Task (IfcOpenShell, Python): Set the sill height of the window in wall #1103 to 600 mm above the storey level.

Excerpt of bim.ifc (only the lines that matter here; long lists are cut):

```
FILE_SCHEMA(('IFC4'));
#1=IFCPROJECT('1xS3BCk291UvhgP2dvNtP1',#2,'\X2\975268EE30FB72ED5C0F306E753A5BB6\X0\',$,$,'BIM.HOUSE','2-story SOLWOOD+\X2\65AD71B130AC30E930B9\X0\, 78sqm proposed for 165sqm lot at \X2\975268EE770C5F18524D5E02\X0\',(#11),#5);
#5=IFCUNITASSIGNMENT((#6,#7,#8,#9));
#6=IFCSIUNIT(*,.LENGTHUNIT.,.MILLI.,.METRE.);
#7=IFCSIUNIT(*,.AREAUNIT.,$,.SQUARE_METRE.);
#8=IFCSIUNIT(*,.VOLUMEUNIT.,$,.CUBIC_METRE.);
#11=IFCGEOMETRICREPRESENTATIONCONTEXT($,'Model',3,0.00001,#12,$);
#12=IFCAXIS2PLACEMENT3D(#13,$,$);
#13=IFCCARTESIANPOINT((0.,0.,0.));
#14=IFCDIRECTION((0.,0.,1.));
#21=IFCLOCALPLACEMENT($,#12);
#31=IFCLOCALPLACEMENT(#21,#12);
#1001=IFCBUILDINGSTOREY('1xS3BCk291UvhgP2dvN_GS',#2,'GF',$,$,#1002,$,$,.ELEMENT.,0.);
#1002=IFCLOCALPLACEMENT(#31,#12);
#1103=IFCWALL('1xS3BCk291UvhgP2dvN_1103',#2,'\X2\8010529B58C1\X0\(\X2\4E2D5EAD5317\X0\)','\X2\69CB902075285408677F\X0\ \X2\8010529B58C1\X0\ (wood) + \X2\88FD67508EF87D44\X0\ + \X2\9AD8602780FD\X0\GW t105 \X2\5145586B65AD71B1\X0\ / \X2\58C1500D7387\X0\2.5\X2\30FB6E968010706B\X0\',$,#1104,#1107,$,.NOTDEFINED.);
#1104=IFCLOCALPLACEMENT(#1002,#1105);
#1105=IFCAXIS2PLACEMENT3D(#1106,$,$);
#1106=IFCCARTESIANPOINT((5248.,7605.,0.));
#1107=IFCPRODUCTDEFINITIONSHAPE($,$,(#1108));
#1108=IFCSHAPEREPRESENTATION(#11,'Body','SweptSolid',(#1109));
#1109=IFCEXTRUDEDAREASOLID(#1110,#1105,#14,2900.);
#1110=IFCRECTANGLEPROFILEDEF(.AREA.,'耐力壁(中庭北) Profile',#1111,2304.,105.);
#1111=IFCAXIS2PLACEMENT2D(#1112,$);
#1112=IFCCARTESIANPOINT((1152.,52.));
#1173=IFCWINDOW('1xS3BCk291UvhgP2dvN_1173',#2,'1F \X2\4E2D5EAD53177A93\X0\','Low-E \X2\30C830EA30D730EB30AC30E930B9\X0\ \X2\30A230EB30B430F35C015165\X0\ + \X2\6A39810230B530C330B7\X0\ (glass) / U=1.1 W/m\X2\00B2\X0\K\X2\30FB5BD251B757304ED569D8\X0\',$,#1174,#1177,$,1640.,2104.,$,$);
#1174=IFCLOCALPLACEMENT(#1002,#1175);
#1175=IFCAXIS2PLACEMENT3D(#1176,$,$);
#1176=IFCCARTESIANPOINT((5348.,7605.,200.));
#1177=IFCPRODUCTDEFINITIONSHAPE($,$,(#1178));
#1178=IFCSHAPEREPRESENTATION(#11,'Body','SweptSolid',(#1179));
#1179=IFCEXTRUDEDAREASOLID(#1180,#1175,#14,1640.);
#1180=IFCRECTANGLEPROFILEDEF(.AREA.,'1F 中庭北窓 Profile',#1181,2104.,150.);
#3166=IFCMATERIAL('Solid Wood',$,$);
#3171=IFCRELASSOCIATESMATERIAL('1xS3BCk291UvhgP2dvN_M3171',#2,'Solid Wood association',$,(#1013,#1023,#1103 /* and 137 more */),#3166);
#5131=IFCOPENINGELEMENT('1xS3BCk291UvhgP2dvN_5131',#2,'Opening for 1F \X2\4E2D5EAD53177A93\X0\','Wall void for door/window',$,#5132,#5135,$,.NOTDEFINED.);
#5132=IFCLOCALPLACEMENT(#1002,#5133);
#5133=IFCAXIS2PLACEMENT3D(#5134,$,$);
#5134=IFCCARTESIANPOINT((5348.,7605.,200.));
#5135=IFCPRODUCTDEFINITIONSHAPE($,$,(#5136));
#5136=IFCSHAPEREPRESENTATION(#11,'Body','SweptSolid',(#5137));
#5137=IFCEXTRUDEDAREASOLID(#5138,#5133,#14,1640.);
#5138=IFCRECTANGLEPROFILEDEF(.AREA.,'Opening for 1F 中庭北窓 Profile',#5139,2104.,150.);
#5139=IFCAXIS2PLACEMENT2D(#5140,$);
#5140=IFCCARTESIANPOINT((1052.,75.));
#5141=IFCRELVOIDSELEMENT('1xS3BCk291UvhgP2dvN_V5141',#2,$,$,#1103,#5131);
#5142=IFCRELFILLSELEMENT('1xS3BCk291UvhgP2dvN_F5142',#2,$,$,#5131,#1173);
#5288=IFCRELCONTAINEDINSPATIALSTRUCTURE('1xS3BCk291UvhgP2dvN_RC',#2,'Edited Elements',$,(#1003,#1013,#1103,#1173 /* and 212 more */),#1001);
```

```python
import numpy as np
import ifcopenshell
import ifcopenshell.api.geometry
import ifcopenshell.geom
import ifcopenshell.util.element
import ifcopenshell.util.placement
import ifcopenshell.util.shape
import ifcopenshell.util.unit

model = ifcopenshell.open("bim.ifc")
unit_scale = ifcopenshell.util.unit.calculate_unit_scale(model)

window = model.by_guid("1xS3BCk291UvhgP2dvN_1173")
opening = window.FillsVoids[0].RelatingOpeningElement
storey = ifcopenshell.util.element.get_container(window, ifc_class="IfcBuildingStorey")
level = ifcopenshell.util.placement.get_local_placement(storey.ObjectPlacement)[2, 3]

# The opening's origin need not be at the sill, so measure its lowest point.
shape = ifcopenshell.geom.create_shape(ifcopenshell.geom.settings(), opening)
bottom = ifcopenshell.util.shape.get_shape_bottom_elevation(shape, shape.geometry) / unit_scale
dz = level + 0.6 / unit_scale - bottom

shift = np.array([0.0, 0.0, dz])
# The window is not placed relative to its opening, so move both.
for product in (opening, window):
    matrix = ifcopenshell.util.placement.get_local_placement(product.ObjectPlacement)
    matrix[:3, 3] += shift
    ifcopenshell.api.geometry.edit_object_placement(model, product=product, matrix=matrix, is_si=False)

print(f"moved by {dz * unit_scale:+.3f} m")

model.write("bim_updated.ifc")
```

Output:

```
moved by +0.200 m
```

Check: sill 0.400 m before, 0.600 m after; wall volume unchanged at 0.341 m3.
